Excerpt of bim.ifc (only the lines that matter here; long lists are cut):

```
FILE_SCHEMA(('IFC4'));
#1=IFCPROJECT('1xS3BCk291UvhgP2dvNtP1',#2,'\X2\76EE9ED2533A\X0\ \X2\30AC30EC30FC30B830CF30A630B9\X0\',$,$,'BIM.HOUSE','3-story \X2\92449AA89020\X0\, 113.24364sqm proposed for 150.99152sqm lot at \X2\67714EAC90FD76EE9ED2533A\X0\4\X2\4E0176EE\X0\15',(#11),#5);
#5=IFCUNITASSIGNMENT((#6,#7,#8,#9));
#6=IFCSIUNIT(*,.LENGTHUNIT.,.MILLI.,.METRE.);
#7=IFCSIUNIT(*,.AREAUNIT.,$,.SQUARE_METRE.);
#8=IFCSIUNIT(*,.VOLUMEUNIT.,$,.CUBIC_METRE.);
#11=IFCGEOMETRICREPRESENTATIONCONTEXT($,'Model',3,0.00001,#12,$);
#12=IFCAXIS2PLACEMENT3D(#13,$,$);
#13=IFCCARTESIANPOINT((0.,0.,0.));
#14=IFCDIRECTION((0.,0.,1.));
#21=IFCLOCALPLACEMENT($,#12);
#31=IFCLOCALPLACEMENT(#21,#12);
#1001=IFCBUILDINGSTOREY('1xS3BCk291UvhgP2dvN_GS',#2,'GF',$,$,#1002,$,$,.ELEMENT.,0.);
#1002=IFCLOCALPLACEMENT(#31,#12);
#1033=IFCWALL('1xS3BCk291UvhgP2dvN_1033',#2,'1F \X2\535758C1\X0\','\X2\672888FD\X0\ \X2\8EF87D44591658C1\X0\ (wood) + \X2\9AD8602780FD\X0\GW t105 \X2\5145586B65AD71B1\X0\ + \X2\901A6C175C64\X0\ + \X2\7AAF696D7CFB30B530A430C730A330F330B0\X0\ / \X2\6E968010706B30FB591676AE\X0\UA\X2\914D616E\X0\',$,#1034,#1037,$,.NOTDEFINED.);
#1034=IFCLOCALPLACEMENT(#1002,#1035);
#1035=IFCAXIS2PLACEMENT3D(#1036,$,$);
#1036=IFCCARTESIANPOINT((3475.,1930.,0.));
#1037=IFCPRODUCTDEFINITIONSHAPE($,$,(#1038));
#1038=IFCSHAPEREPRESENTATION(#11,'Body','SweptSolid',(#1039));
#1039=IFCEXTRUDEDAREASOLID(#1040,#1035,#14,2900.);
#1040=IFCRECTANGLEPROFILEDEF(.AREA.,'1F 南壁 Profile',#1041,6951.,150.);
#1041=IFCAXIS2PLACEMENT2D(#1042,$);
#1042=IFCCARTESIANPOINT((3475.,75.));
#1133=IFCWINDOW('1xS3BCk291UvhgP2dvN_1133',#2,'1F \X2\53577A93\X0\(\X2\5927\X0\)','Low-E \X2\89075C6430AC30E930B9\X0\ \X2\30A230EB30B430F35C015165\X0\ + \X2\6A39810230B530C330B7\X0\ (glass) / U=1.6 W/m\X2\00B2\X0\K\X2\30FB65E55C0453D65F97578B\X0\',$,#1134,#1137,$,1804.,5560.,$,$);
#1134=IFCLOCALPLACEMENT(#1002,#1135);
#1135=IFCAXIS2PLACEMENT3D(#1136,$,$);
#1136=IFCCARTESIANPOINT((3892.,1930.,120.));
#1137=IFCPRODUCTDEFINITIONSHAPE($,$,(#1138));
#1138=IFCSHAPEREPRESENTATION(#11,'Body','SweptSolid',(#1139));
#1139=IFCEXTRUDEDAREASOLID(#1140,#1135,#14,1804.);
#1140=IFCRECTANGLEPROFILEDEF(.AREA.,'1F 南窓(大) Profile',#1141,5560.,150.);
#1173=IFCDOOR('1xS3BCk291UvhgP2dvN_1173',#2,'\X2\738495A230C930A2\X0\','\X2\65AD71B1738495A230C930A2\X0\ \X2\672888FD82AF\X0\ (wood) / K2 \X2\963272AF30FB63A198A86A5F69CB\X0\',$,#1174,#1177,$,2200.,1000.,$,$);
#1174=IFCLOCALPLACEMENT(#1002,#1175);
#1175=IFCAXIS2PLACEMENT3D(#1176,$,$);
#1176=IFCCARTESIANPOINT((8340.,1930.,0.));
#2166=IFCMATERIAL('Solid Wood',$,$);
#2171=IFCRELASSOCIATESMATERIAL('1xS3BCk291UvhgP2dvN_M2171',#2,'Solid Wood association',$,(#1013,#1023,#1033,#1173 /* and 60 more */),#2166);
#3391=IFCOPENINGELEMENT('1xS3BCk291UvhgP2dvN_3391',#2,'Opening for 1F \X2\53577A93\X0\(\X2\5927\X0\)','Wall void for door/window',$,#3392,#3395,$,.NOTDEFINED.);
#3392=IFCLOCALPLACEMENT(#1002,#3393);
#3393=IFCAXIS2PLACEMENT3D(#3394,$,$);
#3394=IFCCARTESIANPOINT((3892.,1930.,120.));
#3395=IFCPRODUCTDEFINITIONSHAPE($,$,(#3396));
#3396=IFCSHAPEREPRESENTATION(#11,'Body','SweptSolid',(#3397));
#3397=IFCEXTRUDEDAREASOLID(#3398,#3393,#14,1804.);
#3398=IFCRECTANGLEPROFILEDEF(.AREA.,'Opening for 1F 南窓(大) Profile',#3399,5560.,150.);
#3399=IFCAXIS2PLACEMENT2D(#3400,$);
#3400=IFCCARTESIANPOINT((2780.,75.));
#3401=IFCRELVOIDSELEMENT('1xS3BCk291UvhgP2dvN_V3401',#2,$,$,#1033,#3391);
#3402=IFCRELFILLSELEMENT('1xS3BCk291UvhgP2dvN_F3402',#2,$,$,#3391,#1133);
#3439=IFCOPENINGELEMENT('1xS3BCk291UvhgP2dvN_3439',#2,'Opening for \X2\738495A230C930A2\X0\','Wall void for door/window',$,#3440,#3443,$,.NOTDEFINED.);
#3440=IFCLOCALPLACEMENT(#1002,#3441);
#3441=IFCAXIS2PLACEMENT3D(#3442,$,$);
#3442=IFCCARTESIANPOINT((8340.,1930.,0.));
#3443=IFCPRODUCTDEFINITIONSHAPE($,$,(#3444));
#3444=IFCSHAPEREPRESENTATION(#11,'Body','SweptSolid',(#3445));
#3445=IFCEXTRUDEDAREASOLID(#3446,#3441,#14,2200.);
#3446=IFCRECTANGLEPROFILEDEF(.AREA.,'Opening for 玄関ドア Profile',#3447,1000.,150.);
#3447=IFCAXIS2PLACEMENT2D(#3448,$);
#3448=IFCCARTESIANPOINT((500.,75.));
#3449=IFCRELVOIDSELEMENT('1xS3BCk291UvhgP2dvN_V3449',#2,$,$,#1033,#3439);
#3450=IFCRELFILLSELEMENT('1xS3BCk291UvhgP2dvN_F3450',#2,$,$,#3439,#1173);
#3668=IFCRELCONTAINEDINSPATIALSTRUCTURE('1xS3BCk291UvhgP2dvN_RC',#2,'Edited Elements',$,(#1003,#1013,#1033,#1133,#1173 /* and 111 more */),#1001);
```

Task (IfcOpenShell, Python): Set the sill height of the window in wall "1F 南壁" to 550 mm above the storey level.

```python
import numpy as np
import ifcopenshell
import ifcopenshell.api.geometry
import ifcopenshell.geom
import ifcopenshell.util.element
import ifcopenshell.util.placement
import ifcopenshell.util.shape
import ifcopenshell.util.unit

model = ifcopenshell.open("bim.ifc")
unit_scale = ifcopenshell.util.unit.calculate_unit_scale(model)

window = model.by_guid("1xS3BCk291UvhgP2dvN_1133")
opening = window.FillsVoids[0].RelatingOpeningElement
storey = ifcopenshell.util.element.get_container(window, ifc_class="IfcBuildingStorey")
level = ifcopenshell.util.placement.get_local_placement(storey.ObjectPlacement)[2, 3]

# The opening's origin need not be at the sill, so measure its lowest point.
shape = ifcopenshell.geom.create_shape(ifcopenshell.geom.settings(), opening)
bottom = ifcopenshell.util.shape.get_shape_bottom_elevation(shape, shape.geometry) / unit_scale
dz = level + 0.55 / unit_scale - bottom

shift = np.array([0.0, 0.0, dz])
# The window is not placed relative to its opening, so move both.
for product in (opening, window):
    matrix = ifcopenshell.util.placement.get_local_placement(product.ObjectPlacement)
    matrix[:3, 3] += shift
    ifcopenshell.api.geometry.edit_object_placement(model, product=product, matrix=matrix, is_si=False)

print(f"moved by {dz * unit_scale:+.3f} m")

model.write("bim-out.ifc")
```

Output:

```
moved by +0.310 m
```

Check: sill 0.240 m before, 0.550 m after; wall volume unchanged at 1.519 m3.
